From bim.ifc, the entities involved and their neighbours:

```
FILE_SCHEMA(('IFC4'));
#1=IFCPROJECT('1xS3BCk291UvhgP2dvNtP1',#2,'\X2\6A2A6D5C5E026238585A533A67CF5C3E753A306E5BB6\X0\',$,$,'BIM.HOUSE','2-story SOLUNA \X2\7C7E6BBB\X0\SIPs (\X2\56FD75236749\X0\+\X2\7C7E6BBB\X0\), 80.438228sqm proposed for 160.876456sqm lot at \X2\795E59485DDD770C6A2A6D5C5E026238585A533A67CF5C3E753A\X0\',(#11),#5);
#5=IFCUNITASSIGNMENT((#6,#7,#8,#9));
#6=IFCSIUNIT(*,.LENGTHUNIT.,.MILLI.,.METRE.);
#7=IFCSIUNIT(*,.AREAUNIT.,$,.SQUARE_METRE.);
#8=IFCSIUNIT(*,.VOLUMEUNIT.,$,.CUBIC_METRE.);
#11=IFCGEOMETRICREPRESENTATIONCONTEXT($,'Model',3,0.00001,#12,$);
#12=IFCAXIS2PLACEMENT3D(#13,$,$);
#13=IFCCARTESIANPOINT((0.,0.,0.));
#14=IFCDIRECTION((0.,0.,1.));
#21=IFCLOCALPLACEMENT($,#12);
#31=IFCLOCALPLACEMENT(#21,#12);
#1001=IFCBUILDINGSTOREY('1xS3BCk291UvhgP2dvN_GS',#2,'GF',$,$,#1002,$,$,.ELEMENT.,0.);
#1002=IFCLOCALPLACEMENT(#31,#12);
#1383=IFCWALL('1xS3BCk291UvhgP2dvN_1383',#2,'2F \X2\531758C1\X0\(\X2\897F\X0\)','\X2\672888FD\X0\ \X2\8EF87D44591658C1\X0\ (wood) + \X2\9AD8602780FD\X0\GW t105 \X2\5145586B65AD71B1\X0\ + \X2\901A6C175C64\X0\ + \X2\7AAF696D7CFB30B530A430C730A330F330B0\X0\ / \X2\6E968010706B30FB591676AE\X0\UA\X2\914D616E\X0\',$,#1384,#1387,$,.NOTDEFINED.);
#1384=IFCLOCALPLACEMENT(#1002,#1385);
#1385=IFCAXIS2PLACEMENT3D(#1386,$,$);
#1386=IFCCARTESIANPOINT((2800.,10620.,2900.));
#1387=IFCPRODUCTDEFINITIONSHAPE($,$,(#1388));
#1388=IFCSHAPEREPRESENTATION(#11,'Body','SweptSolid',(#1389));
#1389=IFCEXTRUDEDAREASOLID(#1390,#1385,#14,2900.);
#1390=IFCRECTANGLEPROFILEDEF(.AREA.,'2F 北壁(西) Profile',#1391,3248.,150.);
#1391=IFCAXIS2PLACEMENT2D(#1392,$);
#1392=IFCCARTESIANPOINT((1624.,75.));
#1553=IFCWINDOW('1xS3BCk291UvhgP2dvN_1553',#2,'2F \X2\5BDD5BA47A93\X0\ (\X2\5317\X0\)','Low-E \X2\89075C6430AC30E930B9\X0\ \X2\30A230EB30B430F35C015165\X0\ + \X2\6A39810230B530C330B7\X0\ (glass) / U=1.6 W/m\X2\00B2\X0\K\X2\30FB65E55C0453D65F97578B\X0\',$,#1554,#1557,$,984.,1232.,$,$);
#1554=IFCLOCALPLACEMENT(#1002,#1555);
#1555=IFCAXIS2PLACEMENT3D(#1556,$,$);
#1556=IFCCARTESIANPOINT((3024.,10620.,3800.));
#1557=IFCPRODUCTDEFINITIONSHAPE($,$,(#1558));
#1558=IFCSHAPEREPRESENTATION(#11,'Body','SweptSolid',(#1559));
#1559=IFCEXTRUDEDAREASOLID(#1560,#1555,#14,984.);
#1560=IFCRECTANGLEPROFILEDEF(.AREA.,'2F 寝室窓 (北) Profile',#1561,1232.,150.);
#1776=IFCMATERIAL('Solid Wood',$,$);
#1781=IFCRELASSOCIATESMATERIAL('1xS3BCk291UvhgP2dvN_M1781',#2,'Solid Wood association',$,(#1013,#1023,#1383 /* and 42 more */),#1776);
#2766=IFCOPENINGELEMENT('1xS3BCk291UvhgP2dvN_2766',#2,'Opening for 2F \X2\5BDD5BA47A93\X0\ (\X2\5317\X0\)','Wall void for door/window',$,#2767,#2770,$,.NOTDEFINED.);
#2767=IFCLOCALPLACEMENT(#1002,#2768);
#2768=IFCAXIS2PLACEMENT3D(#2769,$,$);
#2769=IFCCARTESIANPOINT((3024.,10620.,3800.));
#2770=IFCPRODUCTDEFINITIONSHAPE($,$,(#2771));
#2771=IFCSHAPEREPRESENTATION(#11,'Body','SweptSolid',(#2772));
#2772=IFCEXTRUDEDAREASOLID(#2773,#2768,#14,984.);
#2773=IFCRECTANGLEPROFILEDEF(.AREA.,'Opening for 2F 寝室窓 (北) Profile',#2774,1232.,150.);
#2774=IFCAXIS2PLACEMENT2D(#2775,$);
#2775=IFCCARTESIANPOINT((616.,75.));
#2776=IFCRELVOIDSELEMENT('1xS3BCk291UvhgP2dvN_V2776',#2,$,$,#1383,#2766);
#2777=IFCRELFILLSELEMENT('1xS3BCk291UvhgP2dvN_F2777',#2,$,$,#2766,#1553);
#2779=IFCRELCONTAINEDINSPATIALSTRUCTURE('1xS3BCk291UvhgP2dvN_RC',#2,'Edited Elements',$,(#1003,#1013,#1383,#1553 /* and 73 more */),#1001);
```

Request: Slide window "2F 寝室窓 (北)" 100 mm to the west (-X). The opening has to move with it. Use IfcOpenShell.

```python
import ifcopenshell
import ifcopenshell.api.geometry
import ifcopenshell.util.placement
import ifcopenshell.util.unit

model = ifcopenshell.open("bim.ifc")
unit_scale = ifcopenshell.util.unit.calculate_unit_scale(model)

window = model.by_id(1553)
opening = window.FillsVoids[0].RelatingOpeningElement
wall = opening.VoidsElements[0].RelatingBuildingElement

wall_matrix = ifcopenshell.util.placement.get_local_placement(wall.ObjectPlacement)
shift = wall_matrix[:3, 0] * -0.1 / unit_scale
before = ifcopenshell.util.placement.get_local_placement(window.ObjectPlacement)[:3, 3].copy()

# The window is not placed relative to its opening, so move both.
for product in (opening, window):
    matrix = ifcopenshell.util.placement.get_local_placement(product.ObjectPlacement)
    matrix[:3, 3] += shift
    ifcopenshell.api.geometry.edit_object_placement(model, product=product, matrix=matrix, is_si=False)

after = ifcopenshell.util.placement.get_local_placement(window.ObjectPlacement)[:3, 3]
print("window moved by", (after - before).round(3) + 0.0)

model.write("bim-out.ifc")
```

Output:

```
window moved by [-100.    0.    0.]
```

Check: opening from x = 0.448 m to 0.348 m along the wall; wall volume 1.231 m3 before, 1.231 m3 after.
